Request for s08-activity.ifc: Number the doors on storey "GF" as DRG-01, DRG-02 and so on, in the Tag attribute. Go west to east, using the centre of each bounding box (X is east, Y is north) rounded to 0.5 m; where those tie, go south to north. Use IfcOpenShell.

First a look at what the model holds.

```python
import ifcopenshell
import ifcopenshell.util.element
import ifcopenshell.util.placement

model = ifcopenshell.open("s08-activity.ifc")
print(model.schema)
storey = next(s for s in model.by_type("IfcBuildingStorey") if s.Name == "GF")
doors = [e for e in ifcopenshell.util.element.get_decomposition(storey) if e.is_a("IfcDoor")]
for e in sorted(doors, key=lambda e: e.id()):
    origin = ifcopenshell.util.placement.get_local_placement(e.ObjectPlacement)[:3, 3]
    print(e.id(), e.Tag, e.Name, origin.round(2) + 0.0, sep=" | ")
```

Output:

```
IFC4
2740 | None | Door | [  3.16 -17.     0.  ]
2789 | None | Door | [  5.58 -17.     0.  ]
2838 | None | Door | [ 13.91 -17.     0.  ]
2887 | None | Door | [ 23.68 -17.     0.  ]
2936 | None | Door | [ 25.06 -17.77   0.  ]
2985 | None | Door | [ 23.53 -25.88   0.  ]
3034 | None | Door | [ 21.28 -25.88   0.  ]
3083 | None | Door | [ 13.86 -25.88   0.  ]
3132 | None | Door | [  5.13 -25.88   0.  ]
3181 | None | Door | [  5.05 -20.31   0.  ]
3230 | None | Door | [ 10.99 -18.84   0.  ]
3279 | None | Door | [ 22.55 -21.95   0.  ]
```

```python
import ifcopenshell
import ifcopenshell.geom
import ifcopenshell.util.element
import ifcopenshell.util.shape

model = ifcopenshell.open("s08-activity.ifc")
settings = ifcopenshell.geom.settings()
settings.set("use-world-coords", True)


def centre(element):
    shape = ifcopenshell.geom.create_shape(settings, element)
    return ifcopenshell.util.shape.get_bbox_centroid(shape.geometry)


storey = next(s for s in model.by_type("IfcBuildingStorey") if s.Name == "GF")
doors = [e for e in ifcopenshell.util.element.get_decomposition(storey) if e.is_a("IfcDoor")]

# Insertion points can sit at a corner or the storey origin, so sort by the geometry (in metres).
centres = {e: centre(e) for e in doors}
doors.sort(key=lambda e: (round(centres[e][0] / 0.5), centres[e][1]))

for i, e in enumerate(doors, start=1):
    number = f"DRG-{i:02d}"
    e.Tag = number
    print(e.id(), number)

model.write("s08-activity_rev.ifc")
```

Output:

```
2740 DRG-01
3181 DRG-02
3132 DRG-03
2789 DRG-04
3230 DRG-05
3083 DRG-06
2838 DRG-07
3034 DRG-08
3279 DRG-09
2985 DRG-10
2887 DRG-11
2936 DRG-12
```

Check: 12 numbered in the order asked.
